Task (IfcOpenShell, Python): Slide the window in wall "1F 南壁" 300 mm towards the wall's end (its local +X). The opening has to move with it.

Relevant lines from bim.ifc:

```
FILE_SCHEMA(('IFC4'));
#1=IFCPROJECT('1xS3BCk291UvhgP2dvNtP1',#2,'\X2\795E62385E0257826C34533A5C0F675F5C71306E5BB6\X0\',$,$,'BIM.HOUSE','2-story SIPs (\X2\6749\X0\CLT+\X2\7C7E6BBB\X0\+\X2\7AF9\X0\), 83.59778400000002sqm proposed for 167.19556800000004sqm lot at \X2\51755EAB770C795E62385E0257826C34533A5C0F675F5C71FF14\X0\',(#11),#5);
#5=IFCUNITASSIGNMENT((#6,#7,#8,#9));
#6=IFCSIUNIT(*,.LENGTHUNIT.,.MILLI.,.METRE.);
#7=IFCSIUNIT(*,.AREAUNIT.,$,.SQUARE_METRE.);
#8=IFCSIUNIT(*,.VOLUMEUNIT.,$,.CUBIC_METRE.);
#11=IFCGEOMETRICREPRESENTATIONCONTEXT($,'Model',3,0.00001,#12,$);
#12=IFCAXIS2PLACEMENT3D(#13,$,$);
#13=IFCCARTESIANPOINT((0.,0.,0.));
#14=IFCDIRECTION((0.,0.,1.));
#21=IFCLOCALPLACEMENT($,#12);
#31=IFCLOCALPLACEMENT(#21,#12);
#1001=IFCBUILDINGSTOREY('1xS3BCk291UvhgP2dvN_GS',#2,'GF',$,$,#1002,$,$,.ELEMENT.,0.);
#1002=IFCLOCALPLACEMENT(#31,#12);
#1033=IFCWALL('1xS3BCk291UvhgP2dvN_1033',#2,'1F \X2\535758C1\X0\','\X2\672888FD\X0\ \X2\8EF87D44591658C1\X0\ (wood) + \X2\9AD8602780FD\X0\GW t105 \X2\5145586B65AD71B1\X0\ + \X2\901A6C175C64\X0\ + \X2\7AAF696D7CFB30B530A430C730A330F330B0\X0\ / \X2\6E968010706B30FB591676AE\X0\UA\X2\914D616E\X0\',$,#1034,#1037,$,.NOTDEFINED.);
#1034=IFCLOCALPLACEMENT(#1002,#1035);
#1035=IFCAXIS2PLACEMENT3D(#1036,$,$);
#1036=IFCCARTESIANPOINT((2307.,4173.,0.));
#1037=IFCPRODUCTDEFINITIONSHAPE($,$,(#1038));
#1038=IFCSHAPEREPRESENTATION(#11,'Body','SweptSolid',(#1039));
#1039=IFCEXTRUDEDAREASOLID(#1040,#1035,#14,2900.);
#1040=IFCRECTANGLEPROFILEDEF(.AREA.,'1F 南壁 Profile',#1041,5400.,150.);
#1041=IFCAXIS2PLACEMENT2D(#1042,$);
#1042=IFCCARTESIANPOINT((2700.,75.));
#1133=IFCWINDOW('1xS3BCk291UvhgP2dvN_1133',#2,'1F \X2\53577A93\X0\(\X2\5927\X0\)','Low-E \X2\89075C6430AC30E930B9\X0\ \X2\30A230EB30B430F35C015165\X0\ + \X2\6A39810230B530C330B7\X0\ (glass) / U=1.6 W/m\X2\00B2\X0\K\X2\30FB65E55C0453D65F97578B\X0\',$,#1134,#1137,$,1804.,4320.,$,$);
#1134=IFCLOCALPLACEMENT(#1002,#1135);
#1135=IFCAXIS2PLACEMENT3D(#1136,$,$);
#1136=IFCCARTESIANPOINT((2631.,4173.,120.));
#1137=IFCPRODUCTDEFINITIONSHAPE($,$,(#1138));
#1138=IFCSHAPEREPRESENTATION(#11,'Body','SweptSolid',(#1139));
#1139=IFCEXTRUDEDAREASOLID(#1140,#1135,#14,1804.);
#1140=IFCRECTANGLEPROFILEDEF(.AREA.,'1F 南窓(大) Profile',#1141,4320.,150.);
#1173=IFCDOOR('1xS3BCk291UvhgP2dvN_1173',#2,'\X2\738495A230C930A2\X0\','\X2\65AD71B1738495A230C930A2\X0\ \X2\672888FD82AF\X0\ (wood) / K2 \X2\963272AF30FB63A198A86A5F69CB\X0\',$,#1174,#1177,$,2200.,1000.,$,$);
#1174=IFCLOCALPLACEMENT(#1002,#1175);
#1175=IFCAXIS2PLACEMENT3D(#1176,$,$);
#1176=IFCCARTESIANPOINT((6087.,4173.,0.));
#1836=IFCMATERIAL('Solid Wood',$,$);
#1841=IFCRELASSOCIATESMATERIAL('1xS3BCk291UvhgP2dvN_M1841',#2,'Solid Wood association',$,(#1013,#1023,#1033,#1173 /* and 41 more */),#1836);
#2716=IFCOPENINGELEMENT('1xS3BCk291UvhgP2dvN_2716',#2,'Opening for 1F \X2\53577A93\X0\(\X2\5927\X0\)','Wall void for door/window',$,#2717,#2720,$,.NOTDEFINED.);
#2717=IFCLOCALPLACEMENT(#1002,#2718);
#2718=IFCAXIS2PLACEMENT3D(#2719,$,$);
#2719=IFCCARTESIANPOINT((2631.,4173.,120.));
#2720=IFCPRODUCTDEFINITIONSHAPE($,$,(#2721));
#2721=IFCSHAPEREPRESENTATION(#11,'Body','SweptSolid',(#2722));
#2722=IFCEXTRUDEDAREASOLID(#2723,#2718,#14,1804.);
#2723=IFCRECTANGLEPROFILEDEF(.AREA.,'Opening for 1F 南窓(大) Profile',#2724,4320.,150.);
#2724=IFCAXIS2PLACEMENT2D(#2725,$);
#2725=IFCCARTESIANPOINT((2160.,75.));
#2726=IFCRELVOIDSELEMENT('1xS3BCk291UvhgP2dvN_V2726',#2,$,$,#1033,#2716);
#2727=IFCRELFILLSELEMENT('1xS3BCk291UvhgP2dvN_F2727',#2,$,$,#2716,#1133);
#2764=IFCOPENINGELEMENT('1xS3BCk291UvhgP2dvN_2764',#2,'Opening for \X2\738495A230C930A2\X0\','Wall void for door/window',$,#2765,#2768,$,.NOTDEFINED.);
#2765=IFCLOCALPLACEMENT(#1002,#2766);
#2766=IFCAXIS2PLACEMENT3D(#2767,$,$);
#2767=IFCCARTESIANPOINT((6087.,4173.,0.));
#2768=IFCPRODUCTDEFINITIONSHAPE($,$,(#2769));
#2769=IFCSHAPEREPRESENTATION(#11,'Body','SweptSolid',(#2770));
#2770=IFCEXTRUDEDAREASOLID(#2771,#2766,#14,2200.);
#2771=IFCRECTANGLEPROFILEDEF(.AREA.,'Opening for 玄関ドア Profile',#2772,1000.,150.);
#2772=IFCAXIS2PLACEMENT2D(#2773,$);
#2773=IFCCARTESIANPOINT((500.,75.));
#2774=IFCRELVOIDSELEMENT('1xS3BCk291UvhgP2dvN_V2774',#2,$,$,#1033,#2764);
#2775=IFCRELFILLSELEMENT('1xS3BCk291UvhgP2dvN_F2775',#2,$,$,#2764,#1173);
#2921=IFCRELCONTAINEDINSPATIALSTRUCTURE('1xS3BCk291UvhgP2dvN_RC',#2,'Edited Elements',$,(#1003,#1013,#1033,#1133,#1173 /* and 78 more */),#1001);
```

```python
import ifcopenshell
import ifcopenshell.api.geometry
import ifcopenshell.util.placement
import ifcopenshell.util.unit

model = ifcopenshell.open("bim.ifc")
unit_scale = ifcopenshell.util.unit.calculate_unit_scale(model)

window = model.by_id(1133)
opening = window.FillsVoids[0].RelatingOpeningElement
wall = opening.VoidsElements[0].RelatingBuildingElement

wall_matrix = ifcopenshell.util.placement.get_local_placement(wall.ObjectPlacement)
shift = wall_matrix[:3, 0] * 0.3 / unit_scale
before = ifcopenshell.util.placement.get_local_placement(window.ObjectPlacement)[:3, 3].copy()

# The window is not placed relative to its opening, so move both.
for product in (opening, window):
    matrix = ifcopenshell.util.placement.get_local_placement(product.ObjectPlacement)
    matrix[:3, 3] += shift
    ifcopenshell.api.geometry.edit_object_placement(model, product=product, matrix=matrix, is_si=False)

after = ifcopenshell.util.placement.get_local_placement(window.ObjectPlacement)[:3, 3]
print("window moved by", (after - before).round(3) + 0.0)

model.write("bim_updated.ifc")
```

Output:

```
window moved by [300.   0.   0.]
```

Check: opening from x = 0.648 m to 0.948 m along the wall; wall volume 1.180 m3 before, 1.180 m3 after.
